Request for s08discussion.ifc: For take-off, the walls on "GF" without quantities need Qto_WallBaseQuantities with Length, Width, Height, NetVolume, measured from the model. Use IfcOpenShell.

First a look at what the model holds.

```python
import ifcopenshell
import ifcopenshell.util.element
import ifcopenshell.util.unit

model = ifcopenshell.open("s08discussion.ifc")
print(model.schema)
for unit_type in ("LENGTHUNIT", "AREAUNIT", "VOLUMEUNIT"):
    print(unit_type, ifcopenshell.util.unit.calculate_unit_scale(model, unit_type))
storey = next(s for s in model.by_type("IfcBuildingStorey") if s.Name == "GF")
walls = [e for e in ifcopenshell.util.element.get_decomposition(storey) if e.is_a("IfcWall")]
for e in sorted(walls, key=lambda e: e.id()):
    print(e.id(), e.is_a(), e.Name, list(ifcopenshell.util.element.get_psets(e, qtos_only=True)), sep=" | ")
```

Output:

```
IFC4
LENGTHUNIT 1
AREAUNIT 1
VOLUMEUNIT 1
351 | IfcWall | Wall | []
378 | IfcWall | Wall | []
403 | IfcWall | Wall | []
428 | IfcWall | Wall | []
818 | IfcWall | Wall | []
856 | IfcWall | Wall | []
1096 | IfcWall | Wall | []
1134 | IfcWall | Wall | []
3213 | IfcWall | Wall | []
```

```python
import ifcopenshell
import ifcopenshell.api.pset
import ifcopenshell.geom
import ifcopenshell.util.element
import ifcopenshell.util.shape
import ifcopenshell.util.unit

model = ifcopenshell.open("s08discussion.ifc")
unit_scale = ifcopenshell.util.unit.calculate_unit_scale(model)
volume_scale = ifcopenshell.util.unit.calculate_unit_scale(model, "VOLUMEUNIT")
settings = ifcopenshell.geom.settings()

storey = next(s for s in model.by_type("IfcBuildingStorey") if s.Name == "GF")
walls = [e for e in ifcopenshell.util.element.get_decomposition(storey) if e.is_a("IfcWall")]

for e in sorted(walls, key=lambda e: e.id()):
    if ifcopenshell.util.element.get_psets(e, qtos_only=True, should_inherit=False):
        continue
    # Geometry comes back in metres, in the element's own axes.
    shape = ifcopenshell.geom.create_shape(settings, e)
    values = {
        "Length": ifcopenshell.util.shape.get_x(shape.geometry) / unit_scale,
        "Width": ifcopenshell.util.shape.get_y(shape.geometry) / unit_scale,
        "Height": ifcopenshell.util.shape.get_z(shape.geometry) / unit_scale,
        "NetVolume": ifcopenshell.util.shape.get_volume(shape.geometry) / volume_scale,
    }
    qto = ifcopenshell.api.pset.add_qto(model, product=e, name="Qto_WallBaseQuantities")
    ifcopenshell.api.pset.edit_qto(model, qto=qto, properties=values)
    print(e.id(), {k: round(v, 3) for k, v in values.items()})

model.write("s08discussion_rev.ifc")
```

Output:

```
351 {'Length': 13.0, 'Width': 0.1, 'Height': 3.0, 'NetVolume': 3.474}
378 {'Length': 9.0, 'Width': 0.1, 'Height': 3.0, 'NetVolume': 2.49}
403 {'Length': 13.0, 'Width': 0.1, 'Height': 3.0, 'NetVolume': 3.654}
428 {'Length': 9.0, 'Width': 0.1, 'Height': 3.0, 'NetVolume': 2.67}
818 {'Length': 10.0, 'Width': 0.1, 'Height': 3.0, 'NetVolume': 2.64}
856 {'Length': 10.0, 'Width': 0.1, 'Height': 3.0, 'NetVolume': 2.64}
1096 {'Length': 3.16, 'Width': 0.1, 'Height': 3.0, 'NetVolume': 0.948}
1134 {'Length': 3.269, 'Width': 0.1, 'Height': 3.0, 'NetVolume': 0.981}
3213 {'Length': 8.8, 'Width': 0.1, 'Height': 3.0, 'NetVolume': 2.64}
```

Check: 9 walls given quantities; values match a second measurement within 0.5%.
